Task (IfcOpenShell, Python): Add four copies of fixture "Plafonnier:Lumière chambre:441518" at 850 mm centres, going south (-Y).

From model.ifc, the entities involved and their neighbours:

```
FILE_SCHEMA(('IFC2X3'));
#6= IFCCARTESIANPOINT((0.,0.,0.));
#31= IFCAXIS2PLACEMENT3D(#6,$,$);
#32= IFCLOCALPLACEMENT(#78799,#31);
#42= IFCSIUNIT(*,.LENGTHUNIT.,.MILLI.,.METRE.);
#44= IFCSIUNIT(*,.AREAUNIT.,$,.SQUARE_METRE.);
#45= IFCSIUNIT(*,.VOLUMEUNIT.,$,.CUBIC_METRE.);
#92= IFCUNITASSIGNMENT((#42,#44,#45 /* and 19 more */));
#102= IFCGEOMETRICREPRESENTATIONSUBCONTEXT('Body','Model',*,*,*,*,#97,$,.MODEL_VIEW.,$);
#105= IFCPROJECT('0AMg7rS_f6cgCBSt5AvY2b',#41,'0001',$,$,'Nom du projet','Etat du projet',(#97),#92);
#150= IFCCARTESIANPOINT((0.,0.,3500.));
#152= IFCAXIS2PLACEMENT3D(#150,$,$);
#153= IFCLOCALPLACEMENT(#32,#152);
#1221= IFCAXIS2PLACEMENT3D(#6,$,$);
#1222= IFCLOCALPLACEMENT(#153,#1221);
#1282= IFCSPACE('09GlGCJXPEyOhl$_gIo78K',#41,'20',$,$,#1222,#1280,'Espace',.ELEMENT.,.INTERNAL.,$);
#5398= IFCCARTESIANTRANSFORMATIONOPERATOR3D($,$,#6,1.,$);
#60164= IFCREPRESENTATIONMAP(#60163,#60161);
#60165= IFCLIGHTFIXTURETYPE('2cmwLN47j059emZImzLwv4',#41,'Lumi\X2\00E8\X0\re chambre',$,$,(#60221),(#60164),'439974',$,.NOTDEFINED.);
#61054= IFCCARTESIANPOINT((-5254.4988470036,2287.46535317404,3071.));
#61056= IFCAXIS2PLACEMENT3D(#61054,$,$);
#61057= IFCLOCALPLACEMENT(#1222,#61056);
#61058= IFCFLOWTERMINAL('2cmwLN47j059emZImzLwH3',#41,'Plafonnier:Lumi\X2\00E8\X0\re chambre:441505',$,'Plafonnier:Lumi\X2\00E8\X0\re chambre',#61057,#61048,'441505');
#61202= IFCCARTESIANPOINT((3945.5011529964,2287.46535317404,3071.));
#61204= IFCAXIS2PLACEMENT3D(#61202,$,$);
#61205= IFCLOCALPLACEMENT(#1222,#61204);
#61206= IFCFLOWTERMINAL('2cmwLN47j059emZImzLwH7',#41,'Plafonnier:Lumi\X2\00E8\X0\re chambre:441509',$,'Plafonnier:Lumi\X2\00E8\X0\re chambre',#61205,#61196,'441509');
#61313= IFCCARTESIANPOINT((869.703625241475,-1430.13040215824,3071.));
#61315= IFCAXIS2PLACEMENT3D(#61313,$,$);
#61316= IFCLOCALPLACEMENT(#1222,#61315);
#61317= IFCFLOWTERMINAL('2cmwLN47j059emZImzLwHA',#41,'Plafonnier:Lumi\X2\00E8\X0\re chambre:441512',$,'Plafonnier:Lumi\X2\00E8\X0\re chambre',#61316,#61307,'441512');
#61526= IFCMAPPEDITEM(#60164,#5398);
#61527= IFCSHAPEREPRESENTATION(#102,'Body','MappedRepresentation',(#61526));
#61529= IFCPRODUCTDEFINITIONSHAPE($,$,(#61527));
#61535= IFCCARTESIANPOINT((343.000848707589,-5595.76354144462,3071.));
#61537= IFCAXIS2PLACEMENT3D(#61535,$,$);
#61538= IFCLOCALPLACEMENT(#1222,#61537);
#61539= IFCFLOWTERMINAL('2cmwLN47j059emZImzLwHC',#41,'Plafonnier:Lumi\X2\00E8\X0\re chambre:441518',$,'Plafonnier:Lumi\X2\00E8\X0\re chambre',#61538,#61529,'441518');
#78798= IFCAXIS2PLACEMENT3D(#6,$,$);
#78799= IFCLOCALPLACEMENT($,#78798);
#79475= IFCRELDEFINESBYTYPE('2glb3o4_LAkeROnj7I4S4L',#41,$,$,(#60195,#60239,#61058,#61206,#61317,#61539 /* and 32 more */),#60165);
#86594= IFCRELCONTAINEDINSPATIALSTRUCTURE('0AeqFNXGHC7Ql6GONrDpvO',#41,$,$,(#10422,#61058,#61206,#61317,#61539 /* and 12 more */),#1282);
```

```python
import numpy as np
import ifcopenshell
import ifcopenshell.api.geometry
import ifcopenshell.api.root
import ifcopenshell.util.element
import ifcopenshell.util.placement
import ifcopenshell.util.unit

model = ifcopenshell.open("model.ifc")
unit_scale = ifcopenshell.util.unit.calculate_unit_scale(model)


def reuse_history(source, copy):
    """copy_class also copies each property set's owner history, people and application; keep the originals."""
    for rel in copy.IsDefinedBy:
        if rel.is_a("IfcRelDefinesByProperties") and (history := rel.RelatingPropertyDefinition.OwnerHistory):
            rel.RelatingPropertyDefinition.OwnerHistory = source.OwnerHistory
            ifcopenshell.util.element.remove_deep2(model, history)


source = model.by_guid("2cmwLN47j059emZImzLwHC")
base = ifcopenshell.util.placement.get_local_placement(source.ObjectPlacement)
step = np.array([0.0, -1.0, 0.0]) * 0.85 / unit_scale

for i in range(1, 5):
    copy = ifcopenshell.api.root.copy_class(model, product=source)
    copy.Representation = ifcopenshell.util.element.copy_deep(
        model, source.Representation, exclude=["IfcGeometricRepresentationContext", "IfcRepresentationMap"]
    )
    copy.Name = "Plafonnier:Lumière chambre"
    copy.Tag = None
    reuse_history(source, copy)
    matrix = base.copy()
    matrix[:3, 3] += i * step
    print("added at", matrix[:3, 3].round(3) + 0.0)
    ifcopenshell.api.geometry.edit_object_placement(model, product=copy, matrix=matrix, is_si=False)

model.write("model-out.ifc")
```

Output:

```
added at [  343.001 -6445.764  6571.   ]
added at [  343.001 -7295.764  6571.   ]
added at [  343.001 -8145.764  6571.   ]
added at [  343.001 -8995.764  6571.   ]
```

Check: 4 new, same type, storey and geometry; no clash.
